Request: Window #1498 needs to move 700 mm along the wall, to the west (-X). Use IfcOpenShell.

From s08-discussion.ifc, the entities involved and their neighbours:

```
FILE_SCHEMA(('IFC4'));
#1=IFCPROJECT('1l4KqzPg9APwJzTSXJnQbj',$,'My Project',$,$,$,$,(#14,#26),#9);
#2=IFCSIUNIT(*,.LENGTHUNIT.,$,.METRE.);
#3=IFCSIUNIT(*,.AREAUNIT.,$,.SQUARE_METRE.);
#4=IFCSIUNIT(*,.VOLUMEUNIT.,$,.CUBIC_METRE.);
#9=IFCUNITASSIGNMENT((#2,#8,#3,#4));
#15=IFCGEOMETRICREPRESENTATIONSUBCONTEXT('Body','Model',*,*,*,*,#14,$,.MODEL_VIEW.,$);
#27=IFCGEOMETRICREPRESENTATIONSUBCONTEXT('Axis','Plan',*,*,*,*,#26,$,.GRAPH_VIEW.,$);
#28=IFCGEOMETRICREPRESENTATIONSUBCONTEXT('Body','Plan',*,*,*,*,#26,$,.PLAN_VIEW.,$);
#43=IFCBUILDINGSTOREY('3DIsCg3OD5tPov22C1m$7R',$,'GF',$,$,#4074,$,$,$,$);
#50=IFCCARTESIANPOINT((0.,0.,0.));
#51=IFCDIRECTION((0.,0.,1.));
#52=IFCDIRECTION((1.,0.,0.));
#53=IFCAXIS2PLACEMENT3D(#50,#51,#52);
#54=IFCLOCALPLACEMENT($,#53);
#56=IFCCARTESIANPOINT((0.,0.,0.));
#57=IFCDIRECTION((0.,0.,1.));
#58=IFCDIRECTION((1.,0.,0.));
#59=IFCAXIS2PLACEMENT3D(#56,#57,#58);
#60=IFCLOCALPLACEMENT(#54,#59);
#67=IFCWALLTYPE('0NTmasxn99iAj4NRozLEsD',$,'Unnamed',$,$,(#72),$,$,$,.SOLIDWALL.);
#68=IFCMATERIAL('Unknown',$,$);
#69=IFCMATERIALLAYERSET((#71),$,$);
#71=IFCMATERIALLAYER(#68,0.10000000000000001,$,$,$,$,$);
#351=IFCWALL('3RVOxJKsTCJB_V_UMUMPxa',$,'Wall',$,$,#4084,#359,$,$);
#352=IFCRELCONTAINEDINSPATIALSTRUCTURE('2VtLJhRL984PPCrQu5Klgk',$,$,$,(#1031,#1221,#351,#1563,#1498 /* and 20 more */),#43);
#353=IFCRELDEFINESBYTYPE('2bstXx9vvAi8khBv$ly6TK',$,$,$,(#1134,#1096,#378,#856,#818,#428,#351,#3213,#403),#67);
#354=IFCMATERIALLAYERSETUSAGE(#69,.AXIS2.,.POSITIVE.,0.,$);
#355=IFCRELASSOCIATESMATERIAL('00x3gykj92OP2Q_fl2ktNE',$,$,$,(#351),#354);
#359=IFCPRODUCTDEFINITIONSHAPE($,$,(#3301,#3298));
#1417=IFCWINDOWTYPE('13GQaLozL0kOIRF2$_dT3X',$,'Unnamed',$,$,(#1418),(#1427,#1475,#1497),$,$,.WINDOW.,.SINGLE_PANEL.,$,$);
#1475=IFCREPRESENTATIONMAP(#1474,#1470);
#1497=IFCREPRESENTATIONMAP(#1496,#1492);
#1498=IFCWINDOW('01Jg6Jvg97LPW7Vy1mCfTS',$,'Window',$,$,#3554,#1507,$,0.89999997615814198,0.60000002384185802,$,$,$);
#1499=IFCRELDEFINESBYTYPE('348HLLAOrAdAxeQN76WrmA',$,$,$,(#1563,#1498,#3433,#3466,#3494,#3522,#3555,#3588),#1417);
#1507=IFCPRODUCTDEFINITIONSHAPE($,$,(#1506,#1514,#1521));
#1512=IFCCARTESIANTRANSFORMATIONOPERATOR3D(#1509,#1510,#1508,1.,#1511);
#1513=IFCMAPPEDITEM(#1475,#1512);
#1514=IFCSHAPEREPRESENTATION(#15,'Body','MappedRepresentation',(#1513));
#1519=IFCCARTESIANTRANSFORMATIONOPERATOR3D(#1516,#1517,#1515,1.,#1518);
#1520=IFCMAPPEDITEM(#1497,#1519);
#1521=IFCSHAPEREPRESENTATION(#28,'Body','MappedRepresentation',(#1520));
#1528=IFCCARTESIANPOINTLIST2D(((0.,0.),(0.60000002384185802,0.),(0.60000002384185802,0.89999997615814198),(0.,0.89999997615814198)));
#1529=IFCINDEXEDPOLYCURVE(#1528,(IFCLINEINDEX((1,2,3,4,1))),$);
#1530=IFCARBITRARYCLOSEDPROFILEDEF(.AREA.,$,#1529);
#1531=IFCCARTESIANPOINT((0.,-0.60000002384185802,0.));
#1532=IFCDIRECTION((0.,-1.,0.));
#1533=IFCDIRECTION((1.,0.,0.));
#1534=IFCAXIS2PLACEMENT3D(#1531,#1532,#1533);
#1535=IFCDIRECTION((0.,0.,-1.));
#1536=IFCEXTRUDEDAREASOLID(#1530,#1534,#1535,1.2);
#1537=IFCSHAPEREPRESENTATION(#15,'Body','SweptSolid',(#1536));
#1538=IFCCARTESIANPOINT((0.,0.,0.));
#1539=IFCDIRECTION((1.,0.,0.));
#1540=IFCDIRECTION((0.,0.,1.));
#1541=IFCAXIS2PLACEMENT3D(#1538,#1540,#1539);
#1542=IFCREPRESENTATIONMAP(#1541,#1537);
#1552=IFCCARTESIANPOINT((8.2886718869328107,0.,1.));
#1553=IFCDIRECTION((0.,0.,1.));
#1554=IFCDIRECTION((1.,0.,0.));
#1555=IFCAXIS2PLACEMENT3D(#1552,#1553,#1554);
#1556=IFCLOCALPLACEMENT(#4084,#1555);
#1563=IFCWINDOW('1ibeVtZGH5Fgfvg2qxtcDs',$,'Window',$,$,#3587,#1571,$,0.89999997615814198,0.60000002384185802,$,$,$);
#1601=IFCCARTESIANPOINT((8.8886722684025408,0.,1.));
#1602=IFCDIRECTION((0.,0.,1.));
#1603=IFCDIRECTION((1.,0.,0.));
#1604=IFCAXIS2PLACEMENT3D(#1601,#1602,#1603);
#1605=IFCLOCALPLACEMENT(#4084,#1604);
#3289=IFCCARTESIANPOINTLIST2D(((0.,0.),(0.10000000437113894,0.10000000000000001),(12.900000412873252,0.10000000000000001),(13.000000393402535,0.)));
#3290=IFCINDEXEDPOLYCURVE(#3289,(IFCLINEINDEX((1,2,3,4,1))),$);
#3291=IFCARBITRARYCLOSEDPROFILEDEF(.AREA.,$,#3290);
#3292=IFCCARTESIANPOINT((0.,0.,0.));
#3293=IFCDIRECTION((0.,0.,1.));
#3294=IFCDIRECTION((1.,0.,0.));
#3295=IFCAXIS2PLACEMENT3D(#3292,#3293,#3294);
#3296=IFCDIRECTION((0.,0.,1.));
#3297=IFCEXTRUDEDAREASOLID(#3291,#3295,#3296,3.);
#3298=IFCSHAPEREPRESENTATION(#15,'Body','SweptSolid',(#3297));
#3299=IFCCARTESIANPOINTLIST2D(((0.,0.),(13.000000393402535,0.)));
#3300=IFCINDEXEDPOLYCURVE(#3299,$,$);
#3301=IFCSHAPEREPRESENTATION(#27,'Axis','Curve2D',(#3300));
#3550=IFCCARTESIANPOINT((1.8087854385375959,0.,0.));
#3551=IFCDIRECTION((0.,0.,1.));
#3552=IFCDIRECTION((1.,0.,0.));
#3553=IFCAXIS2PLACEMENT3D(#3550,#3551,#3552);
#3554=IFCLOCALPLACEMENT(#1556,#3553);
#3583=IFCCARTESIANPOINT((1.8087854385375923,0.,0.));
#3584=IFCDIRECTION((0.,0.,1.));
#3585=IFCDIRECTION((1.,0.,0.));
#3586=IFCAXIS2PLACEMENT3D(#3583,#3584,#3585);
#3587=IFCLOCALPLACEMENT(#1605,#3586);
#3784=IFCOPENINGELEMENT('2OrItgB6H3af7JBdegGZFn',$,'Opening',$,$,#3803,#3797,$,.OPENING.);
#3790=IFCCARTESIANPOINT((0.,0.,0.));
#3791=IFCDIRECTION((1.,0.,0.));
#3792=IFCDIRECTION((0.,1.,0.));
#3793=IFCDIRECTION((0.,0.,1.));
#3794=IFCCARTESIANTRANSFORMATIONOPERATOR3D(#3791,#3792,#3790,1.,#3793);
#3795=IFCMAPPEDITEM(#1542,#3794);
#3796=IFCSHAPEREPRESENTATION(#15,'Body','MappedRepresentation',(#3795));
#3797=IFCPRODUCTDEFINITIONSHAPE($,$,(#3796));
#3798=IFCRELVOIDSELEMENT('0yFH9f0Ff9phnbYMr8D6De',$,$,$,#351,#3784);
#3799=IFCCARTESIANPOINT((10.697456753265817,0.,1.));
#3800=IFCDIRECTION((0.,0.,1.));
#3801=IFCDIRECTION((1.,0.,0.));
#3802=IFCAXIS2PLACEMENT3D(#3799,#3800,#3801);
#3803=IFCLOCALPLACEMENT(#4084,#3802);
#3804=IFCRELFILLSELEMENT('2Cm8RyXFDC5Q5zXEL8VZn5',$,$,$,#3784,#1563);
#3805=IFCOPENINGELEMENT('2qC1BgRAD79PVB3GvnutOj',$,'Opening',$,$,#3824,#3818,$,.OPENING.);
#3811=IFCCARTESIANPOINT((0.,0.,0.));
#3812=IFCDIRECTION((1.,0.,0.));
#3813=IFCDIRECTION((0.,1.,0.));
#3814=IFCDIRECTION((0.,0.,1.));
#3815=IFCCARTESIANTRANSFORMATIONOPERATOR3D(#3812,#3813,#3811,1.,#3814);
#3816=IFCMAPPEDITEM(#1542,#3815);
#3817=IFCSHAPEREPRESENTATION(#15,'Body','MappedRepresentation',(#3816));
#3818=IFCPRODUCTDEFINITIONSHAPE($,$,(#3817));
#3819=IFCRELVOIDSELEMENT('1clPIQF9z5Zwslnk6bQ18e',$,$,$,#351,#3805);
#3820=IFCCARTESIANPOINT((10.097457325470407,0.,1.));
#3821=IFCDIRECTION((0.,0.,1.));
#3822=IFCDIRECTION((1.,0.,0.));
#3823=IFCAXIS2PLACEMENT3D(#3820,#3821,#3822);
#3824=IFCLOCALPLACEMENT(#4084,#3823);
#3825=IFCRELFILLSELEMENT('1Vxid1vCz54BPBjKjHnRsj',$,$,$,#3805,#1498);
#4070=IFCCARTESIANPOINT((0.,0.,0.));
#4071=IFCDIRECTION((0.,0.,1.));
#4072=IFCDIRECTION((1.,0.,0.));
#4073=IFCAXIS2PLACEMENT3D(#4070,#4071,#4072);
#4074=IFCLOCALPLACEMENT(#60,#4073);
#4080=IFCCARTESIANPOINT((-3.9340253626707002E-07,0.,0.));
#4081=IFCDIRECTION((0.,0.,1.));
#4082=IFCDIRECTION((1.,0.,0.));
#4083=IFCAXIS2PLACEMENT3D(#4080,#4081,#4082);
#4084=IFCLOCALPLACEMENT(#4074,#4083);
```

```python
import ifcopenshell
import ifcopenshell.api.geometry
import ifcopenshell.util.placement

model = ifcopenshell.open("s08-discussion.ifc")

window = model.by_guid("01Jg6Jvg97LPW7Vy1mCfTS")
opening = window.FillsVoids[0].RelatingOpeningElement
wall = opening.VoidsElements[0].RelatingBuildingElement

wall_matrix = ifcopenshell.util.placement.get_local_placement(wall.ObjectPlacement)
shift = wall_matrix[:3, 0] * -0.7
before = ifcopenshell.util.placement.get_local_placement(window.ObjectPlacement)[:3, 3].copy()

# The window is not placed relative to its opening, so move both.
for product in (opening, window):
    matrix = ifcopenshell.util.placement.get_local_placement(product.ObjectPlacement)
    matrix[:3, 3] += shift
    ifcopenshell.api.geometry.edit_object_placement(model, product=product, matrix=matrix, is_si=False)

after = ifcopenshell.util.placement.get_local_placement(window.ObjectPlacement)[:3, 3]
print("window moved by", (after - before).round(3) + 0.0)

model.write("s08-discussion_rev.ifc")
```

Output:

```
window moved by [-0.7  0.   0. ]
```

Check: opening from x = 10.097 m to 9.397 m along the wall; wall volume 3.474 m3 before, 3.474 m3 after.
